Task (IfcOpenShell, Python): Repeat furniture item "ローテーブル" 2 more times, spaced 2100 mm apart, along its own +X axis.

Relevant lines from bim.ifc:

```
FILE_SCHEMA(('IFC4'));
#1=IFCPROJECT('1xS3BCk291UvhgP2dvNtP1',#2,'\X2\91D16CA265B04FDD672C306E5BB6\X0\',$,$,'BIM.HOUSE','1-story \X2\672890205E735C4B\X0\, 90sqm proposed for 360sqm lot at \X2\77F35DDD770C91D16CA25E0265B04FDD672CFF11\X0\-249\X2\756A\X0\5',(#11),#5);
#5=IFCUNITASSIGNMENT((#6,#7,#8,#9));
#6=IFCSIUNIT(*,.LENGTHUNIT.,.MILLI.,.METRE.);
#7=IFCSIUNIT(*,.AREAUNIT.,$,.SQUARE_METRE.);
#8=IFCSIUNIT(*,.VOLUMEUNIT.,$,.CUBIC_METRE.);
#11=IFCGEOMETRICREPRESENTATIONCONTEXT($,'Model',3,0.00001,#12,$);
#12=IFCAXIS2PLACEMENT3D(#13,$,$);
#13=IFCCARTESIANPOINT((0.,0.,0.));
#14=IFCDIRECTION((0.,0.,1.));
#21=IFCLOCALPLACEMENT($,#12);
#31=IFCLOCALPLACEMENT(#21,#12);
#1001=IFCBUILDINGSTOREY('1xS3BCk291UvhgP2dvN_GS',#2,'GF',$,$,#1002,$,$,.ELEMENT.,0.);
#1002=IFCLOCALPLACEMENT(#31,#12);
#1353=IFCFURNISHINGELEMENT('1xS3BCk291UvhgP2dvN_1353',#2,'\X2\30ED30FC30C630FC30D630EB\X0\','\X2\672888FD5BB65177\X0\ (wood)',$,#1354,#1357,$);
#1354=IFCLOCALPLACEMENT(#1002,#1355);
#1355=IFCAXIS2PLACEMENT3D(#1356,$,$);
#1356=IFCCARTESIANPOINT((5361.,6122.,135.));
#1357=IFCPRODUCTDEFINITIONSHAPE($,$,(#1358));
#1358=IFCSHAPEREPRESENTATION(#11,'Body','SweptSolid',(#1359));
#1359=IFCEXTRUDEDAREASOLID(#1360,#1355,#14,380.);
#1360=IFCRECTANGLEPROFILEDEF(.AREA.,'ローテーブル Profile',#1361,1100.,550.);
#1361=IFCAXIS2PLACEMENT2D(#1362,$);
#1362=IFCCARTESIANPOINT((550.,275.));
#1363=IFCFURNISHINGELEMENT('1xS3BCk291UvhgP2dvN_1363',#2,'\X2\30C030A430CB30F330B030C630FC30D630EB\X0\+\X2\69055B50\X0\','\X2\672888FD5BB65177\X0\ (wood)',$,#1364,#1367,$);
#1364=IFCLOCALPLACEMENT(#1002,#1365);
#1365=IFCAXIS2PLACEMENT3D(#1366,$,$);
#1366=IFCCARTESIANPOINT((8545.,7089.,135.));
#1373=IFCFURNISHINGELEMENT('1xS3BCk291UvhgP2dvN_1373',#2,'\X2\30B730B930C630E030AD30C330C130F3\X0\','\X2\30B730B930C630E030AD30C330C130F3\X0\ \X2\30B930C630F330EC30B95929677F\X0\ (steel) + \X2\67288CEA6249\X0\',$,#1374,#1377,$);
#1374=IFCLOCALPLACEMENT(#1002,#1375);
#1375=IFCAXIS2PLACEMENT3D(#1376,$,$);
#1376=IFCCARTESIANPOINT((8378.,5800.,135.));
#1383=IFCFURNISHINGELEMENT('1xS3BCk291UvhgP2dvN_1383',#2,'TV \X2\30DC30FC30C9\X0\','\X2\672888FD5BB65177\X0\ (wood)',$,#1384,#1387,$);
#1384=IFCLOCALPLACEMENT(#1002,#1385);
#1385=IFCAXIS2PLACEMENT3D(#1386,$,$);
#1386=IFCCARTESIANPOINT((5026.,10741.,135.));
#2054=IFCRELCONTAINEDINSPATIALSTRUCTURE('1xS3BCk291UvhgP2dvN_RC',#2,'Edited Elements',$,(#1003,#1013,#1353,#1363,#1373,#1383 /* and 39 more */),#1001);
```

```python
import ifcopenshell
import ifcopenshell.api.geometry
import ifcopenshell.api.root
import ifcopenshell.util.element
import ifcopenshell.util.placement
import ifcopenshell.util.unit

model = ifcopenshell.open("bim.ifc")
unit_scale = ifcopenshell.util.unit.calculate_unit_scale(model)


def reuse_history(source, copy):
    """copy_class also copies each property set's owner history, people and application; keep the originals."""
    for rel in copy.IsDefinedBy:
        if rel.is_a("IfcRelDefinesByProperties") and (history := rel.RelatingPropertyDefinition.OwnerHistory):
            rel.RelatingPropertyDefinition.OwnerHistory = source.OwnerHistory
            ifcopenshell.util.element.remove_deep2(model, history)


source = model.by_guid("1xS3BCk291UvhgP2dvN_1353")
base = ifcopenshell.util.placement.get_local_placement(source.ObjectPlacement)
step = base[:3, 0] * 2.1 / unit_scale

for i in range(1, 3):
    copy = ifcopenshell.api.root.copy_class(model, product=source)
    copy.Representation = ifcopenshell.util.element.copy_deep(
        model, source.Representation, exclude=["IfcGeometricRepresentationContext", "IfcRepresentationMap"]
    )
    reuse_history(source, copy)
    matrix = base.copy()
    matrix[:3, 3] += i * step
    print("added at", matrix[:3, 3].round(3) + 0.0)
    ifcopenshell.api.geometry.edit_object_placement(model, product=copy, matrix=matrix, is_si=False)

model.write("bim_updated.ifc")
```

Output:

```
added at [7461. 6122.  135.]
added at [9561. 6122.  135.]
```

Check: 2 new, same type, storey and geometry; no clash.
